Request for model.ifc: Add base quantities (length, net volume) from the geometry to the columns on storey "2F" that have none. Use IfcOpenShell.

First a look at what the model holds.

```python
import ifcopenshell
import ifcopenshell.util.element
import ifcopenshell.util.unit

model = ifcopenshell.open("model.ifc")
print(model.schema)
for unit_type in ("LENGTHUNIT", "AREAUNIT", "VOLUMEUNIT"):
    print(unit_type, ifcopenshell.util.unit.calculate_unit_scale(model, unit_type))
storey = next(s for s in model.by_type("IfcBuildingStorey") if s.Name == "2F")
columns = [e for e in ifcopenshell.util.element.get_decomposition(storey) if e.is_a("IfcColumn")]
for e in sorted(columns, key=lambda e: e.id()):
    print(e.id(), e.is_a(), e.Name, list(ifcopenshell.util.element.get_psets(e, qtos_only=True)), sep=" | ")
```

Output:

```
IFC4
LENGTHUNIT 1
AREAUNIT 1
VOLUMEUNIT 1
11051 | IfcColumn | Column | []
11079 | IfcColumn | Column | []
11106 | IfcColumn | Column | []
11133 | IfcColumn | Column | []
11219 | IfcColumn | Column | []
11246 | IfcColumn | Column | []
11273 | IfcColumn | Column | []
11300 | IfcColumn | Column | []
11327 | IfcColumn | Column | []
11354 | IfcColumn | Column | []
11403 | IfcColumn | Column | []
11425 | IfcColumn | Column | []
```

```python
import ifcopenshell
import ifcopenshell.api.pset
import ifcopenshell.geom
import ifcopenshell.util.element
import ifcopenshell.util.shape
import ifcopenshell.util.unit

model = ifcopenshell.open("model.ifc")
unit_scale = ifcopenshell.util.unit.calculate_unit_scale(model)
volume_scale = ifcopenshell.util.unit.calculate_unit_scale(model, "VOLUMEUNIT")
settings = ifcopenshell.geom.settings()

storey = next(s for s in model.by_type("IfcBuildingStorey") if s.Name == "2F")
columns = [e for e in ifcopenshell.util.element.get_decomposition(storey) if e.is_a("IfcColumn")]

for e in sorted(columns, key=lambda e: e.id()):
    if ifcopenshell.util.element.get_psets(e, qtos_only=True, should_inherit=False):
        continue
    # Geometry comes back in metres, in the element's own axes.
    shape = ifcopenshell.geom.create_shape(settings, e)
    values = {
        "Length": ifcopenshell.util.shape.get_z(shape.geometry) / unit_scale,
        "NetVolume": ifcopenshell.util.shape.get_volume(shape.geometry) / volume_scale,
    }
    qto = ifcopenshell.api.pset.add_qto(model, product=e, name="Qto_ColumnBaseQuantities")
    ifcopenshell.api.pset.edit_qto(model, qto=qto, properties=values)
    print(e.id(), {k: round(v, 3) for k, v in values.items()})

model.write("model_v2.ifc")
```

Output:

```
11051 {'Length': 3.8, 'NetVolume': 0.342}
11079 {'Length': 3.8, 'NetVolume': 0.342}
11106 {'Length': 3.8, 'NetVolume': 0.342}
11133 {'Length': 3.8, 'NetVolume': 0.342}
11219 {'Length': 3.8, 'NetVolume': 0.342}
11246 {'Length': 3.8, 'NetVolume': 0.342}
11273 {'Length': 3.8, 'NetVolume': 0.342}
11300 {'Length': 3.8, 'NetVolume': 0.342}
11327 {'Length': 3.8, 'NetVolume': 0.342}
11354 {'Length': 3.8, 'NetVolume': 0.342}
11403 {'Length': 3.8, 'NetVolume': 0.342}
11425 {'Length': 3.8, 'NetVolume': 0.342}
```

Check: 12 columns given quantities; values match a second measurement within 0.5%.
